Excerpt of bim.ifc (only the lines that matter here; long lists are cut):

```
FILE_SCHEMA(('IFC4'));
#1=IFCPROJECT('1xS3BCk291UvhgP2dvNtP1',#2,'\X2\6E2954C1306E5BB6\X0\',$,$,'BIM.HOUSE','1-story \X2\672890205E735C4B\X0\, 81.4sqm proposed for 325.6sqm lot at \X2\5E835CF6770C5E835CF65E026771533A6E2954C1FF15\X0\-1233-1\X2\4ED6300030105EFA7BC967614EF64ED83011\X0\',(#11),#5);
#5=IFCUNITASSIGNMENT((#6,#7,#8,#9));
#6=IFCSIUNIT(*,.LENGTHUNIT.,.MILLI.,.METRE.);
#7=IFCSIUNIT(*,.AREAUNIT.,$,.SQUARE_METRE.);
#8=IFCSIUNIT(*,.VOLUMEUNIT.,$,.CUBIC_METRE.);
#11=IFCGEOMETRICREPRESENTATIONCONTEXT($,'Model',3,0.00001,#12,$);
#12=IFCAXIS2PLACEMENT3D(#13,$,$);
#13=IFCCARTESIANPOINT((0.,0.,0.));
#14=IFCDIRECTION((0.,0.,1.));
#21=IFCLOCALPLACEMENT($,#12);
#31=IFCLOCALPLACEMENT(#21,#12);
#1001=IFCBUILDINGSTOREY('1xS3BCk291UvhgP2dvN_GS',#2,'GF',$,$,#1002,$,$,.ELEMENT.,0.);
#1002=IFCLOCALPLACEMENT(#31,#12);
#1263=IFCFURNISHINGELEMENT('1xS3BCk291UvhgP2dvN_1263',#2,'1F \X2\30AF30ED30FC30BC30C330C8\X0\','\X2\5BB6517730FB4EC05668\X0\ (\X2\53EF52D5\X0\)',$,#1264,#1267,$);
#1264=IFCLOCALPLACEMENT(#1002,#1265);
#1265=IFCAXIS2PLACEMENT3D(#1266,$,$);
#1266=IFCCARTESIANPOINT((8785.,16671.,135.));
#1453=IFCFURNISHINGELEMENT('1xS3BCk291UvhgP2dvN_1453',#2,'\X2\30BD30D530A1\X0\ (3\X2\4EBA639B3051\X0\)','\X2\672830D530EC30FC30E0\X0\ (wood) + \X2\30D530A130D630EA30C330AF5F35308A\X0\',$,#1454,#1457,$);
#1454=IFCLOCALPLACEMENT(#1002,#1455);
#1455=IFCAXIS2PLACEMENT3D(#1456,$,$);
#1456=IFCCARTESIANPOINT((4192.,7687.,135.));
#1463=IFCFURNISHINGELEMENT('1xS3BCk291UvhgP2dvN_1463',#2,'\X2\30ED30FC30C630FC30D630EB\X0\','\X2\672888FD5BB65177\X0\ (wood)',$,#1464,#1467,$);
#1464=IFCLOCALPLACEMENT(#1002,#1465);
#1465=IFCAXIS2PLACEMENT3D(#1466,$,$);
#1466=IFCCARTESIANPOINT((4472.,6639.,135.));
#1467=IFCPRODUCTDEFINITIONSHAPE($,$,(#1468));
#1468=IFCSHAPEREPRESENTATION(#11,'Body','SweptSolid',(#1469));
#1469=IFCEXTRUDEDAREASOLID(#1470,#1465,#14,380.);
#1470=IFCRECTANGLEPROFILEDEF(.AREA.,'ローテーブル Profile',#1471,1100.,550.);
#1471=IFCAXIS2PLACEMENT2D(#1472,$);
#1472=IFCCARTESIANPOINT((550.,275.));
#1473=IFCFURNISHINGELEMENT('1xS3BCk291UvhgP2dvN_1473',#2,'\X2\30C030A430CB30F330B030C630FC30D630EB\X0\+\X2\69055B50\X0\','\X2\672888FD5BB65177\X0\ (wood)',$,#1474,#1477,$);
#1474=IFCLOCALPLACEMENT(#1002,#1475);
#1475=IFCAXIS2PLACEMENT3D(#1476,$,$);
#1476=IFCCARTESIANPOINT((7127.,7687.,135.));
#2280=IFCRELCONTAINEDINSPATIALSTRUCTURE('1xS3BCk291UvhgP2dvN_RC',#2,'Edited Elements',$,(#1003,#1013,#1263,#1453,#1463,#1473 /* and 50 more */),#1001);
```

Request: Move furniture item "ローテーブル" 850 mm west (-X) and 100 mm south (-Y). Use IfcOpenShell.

```python
import ifcopenshell
import ifcopenshell.api.geometry
import ifcopenshell.util.placement
import ifcopenshell.util.unit

model = ifcopenshell.open("bim.ifc")
unit_scale = ifcopenshell.util.unit.calculate_unit_scale(model)

item = model.by_id(1463)
matrix = ifcopenshell.util.placement.get_local_placement(item.ObjectPlacement)
matrix[0, 3] -= 0.85 / unit_scale
matrix[1, 3] -= 0.1 / unit_scale
ifcopenshell.api.geometry.edit_object_placement(model, product=item, matrix=matrix, is_si=False)

print(ifcopenshell.util.placement.get_local_placement(item.ObjectPlacement).round(3) + 0.0)

model.write("bim_updated.ifc")
```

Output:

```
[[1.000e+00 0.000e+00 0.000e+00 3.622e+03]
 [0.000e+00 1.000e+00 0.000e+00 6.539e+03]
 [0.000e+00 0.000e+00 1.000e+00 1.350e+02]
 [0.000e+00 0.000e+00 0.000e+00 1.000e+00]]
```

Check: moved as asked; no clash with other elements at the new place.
